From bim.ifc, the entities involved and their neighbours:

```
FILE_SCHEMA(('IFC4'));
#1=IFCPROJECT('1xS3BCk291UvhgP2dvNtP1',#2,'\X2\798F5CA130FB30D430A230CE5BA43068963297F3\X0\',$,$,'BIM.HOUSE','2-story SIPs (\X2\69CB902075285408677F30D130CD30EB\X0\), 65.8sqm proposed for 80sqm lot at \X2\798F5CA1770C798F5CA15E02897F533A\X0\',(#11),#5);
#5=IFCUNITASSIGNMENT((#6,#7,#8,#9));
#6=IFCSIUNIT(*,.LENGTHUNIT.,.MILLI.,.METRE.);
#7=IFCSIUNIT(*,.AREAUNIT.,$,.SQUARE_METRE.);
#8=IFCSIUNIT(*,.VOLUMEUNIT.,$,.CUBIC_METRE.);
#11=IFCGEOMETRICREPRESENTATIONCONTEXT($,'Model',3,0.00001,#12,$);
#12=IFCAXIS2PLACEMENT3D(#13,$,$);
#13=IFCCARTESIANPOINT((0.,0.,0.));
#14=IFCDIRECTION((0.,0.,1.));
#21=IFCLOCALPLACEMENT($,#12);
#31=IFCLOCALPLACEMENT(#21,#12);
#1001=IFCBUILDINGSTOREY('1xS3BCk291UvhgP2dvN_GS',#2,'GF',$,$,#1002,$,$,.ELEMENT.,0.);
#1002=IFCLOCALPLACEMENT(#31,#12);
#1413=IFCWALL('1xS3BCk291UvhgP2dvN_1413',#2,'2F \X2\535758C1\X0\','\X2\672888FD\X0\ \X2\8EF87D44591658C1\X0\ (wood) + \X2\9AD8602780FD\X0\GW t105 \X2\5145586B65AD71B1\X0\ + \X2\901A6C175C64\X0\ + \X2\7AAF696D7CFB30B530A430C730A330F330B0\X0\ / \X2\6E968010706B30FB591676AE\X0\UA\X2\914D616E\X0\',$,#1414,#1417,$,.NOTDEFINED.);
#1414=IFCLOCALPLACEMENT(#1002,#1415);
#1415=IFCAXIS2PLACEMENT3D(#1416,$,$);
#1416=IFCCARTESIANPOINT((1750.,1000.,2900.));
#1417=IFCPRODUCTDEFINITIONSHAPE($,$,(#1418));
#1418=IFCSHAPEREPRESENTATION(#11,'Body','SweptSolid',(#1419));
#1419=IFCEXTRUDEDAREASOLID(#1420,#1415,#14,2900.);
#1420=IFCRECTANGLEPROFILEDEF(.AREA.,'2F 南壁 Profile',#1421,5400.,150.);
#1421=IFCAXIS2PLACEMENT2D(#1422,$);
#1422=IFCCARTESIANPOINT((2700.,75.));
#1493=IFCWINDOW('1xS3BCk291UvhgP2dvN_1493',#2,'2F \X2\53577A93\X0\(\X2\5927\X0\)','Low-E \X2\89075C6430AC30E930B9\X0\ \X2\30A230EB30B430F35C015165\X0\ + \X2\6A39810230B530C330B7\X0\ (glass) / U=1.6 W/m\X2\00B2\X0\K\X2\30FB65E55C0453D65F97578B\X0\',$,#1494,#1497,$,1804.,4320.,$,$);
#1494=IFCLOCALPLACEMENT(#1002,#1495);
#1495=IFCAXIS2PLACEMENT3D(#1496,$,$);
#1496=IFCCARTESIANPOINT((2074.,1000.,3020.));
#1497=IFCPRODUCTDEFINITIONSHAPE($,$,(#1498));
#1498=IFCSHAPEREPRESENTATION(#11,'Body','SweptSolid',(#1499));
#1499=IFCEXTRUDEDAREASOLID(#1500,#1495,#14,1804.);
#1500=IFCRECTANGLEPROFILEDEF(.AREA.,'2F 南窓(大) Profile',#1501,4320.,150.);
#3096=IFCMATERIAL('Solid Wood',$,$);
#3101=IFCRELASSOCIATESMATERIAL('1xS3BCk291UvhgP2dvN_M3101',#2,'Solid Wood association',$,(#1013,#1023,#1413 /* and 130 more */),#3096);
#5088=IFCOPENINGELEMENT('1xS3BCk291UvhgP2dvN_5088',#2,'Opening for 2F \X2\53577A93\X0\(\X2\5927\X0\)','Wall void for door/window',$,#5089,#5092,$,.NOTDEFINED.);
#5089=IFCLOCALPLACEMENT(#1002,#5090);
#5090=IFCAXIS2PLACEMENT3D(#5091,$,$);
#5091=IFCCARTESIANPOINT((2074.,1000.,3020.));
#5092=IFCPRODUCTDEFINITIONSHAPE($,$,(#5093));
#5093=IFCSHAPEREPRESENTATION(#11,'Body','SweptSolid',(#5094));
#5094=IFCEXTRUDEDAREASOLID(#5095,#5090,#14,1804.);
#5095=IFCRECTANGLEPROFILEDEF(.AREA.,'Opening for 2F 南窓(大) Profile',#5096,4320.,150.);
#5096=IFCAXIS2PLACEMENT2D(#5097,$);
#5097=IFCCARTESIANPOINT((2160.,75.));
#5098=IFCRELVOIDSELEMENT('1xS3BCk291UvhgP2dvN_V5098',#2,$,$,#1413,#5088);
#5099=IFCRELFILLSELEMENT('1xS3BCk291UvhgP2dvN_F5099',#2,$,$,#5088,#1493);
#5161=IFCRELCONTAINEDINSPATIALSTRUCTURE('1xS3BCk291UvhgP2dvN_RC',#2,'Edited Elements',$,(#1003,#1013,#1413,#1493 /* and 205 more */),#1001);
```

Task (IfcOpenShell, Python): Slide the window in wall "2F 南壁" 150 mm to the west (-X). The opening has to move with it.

```python
import ifcopenshell
import ifcopenshell.api.geometry
import ifcopenshell.util.placement

model = ifcopenshell.open("bim.ifc")

window = model.by_guid("1xS3BCk291UvhgP2dvN_1493")
opening = window.FillsVoids[0].RelatingOpeningElement
wall = opening.VoidsElements[0].RelatingBuildingElement

wall_matrix = ifcopenshell.util.placement.get_local_placement(wall.ObjectPlacement)
shift = wall_matrix[:3, 0] * -150.0
before = ifcopenshell.util.placement.get_local_placement(window.ObjectPlacement)[:3, 3].copy()

# The window is not placed relative to its opening, so move both.
for product in (opening, window):
    matrix = ifcopenshell.util.placement.get_local_placement(product.ObjectPlacement)
    matrix[:3, 3] += shift
    ifcopenshell.api.geometry.edit_object_placement(model, product=product, matrix=matrix, is_si=False)

after = ifcopenshell.util.placement.get_local_placement(window.ObjectPlacement)[:3, 3]
print("window moved by", (after - before).round(3) + 0.0)

model.write("bim_updated.ifc")
```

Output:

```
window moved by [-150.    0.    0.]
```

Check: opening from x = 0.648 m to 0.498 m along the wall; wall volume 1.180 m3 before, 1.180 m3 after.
